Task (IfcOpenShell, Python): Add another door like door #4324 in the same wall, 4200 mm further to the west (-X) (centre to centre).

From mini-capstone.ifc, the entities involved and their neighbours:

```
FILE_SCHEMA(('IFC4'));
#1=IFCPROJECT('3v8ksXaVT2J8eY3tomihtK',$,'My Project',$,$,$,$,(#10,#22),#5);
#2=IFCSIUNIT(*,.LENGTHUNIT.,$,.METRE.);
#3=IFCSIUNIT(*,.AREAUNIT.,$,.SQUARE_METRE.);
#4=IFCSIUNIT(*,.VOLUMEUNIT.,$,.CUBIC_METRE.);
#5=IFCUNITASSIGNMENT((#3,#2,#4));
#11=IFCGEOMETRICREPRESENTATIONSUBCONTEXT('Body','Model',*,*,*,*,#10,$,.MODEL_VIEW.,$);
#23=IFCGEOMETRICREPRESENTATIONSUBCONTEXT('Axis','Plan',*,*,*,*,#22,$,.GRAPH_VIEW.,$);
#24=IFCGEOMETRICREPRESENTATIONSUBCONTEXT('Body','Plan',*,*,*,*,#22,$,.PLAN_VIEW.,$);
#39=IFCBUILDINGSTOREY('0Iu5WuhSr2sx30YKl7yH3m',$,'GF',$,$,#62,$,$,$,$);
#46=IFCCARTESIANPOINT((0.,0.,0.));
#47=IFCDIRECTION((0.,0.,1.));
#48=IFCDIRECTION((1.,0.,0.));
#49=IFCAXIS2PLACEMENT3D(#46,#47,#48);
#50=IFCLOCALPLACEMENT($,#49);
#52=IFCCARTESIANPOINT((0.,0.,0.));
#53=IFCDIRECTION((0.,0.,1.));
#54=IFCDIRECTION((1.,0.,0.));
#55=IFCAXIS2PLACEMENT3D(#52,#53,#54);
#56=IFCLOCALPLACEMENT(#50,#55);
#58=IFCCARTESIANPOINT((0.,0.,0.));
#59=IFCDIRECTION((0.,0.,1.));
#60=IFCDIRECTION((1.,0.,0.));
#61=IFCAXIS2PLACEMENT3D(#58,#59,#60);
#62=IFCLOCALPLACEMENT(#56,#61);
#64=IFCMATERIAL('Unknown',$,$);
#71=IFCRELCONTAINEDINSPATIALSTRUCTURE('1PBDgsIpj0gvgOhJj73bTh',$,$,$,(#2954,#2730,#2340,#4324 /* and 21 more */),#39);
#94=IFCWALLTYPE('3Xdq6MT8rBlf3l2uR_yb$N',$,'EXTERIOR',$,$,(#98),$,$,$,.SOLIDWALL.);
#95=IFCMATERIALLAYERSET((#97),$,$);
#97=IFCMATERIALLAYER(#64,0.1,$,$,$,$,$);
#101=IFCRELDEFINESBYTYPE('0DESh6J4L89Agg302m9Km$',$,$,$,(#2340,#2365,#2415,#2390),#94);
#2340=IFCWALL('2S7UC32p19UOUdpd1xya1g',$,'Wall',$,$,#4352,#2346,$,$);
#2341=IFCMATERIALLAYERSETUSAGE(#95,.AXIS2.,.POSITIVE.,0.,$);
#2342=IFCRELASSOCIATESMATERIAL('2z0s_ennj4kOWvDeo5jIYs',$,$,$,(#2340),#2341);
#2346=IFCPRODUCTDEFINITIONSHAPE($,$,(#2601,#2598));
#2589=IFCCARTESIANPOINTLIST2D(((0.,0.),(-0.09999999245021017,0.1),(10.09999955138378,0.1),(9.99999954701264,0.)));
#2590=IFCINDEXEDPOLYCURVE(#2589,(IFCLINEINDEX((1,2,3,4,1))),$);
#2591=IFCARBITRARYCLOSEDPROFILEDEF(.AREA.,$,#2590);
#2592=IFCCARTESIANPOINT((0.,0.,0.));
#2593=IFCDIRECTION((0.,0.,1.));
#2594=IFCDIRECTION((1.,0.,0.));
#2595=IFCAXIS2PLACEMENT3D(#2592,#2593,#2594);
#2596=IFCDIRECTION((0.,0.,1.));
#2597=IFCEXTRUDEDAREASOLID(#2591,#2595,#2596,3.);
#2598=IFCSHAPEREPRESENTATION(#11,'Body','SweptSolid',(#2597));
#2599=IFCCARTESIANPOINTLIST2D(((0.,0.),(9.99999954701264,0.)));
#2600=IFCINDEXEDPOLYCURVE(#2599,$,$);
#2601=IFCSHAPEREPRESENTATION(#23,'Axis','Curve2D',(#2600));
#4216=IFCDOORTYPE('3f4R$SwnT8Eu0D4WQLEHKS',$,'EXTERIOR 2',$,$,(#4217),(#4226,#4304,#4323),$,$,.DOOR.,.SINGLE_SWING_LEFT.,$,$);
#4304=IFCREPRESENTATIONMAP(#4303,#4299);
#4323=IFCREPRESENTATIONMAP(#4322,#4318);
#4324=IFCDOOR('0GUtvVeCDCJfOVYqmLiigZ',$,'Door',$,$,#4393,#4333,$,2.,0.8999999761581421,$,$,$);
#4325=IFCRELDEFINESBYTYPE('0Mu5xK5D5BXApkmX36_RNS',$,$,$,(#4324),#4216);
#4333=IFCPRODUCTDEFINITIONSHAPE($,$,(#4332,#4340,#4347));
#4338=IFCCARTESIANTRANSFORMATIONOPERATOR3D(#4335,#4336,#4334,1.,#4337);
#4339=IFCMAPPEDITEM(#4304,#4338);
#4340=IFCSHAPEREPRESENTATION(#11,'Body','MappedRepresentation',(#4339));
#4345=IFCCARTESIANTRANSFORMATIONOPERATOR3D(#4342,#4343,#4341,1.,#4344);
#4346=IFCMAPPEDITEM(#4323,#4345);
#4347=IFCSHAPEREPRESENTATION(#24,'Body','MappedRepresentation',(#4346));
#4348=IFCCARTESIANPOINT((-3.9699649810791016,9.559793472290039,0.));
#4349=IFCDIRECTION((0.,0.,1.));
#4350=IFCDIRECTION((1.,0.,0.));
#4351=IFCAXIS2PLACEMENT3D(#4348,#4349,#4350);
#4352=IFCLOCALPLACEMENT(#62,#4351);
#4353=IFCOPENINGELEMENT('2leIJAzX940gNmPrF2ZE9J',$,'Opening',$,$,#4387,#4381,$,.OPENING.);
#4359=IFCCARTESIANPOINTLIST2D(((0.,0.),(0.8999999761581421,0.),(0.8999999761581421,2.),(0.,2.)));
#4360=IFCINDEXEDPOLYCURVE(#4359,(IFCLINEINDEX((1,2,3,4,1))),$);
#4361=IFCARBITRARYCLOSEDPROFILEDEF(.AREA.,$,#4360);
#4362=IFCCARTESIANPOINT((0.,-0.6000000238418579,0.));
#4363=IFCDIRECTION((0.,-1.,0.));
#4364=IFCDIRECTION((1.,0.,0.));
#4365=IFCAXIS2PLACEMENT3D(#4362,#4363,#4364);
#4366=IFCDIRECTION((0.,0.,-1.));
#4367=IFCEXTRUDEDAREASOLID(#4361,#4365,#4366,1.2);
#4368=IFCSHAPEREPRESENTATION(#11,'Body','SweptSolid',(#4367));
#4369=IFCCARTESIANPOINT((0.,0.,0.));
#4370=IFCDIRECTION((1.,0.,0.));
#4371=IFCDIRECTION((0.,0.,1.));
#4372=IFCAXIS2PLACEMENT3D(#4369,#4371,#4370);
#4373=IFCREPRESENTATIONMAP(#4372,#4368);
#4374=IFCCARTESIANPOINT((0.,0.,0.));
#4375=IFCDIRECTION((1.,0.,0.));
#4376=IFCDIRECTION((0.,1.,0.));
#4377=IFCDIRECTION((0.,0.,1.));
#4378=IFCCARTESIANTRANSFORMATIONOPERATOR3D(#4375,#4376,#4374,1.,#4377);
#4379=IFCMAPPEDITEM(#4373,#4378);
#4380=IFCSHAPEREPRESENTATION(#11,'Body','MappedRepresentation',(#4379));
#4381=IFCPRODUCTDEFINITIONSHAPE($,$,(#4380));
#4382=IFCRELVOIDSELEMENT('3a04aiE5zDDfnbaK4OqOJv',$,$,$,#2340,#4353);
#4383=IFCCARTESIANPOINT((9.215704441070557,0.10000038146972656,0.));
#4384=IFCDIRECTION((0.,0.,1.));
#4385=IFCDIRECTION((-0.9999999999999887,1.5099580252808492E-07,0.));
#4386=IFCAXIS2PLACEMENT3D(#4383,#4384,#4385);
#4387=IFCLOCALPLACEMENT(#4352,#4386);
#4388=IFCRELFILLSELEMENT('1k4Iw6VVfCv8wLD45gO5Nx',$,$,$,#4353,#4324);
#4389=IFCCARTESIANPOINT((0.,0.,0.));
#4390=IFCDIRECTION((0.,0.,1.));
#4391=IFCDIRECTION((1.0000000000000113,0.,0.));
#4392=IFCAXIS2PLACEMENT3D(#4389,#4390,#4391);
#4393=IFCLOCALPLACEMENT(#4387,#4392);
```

```python
import ifcopenshell
import ifcopenshell.api.feature
import ifcopenshell.api.geometry
import ifcopenshell.api.root
import ifcopenshell.geom
import ifcopenshell.util.element
import ifcopenshell.util.placement
import ifcopenshell.util.shape

model = ifcopenshell.open("mini-capstone.ifc")
settings = ifcopenshell.geom.settings()


def volume(element):
    """Net volume in cubic metres, openings subtracted."""
    shape = ifcopenshell.geom.create_shape(settings, element)
    return ifcopenshell.util.shape.get_volume(shape.geometry)


door = model.by_id(4324)
opening = door.FillsVoids[0].RelatingOpeningElement
wall = opening.VoidsElements[0].RelatingBuildingElement
before = volume(wall)
shift = ifcopenshell.util.placement.get_local_placement(wall.ObjectPlacement)[:3, 0] * -4.2

# copy_class copies the void relationship, type, container and properties, but no geometry.
new_opening = ifcopenshell.api.root.copy_class(model, product=opening)
new_opening.Representation = ifcopenshell.util.element.copy_deep(
    model, opening.Representation, exclude=["IfcGeometricRepresentationContext", "IfcRepresentationMap"]
)
new_door = ifcopenshell.api.root.copy_class(model, product=door)
new_door.Representation = ifcopenshell.util.element.copy_deep(
    model, door.Representation, exclude=["IfcGeometricRepresentationContext", "IfcRepresentationMap"]
)
ifcopenshell.api.feature.add_filling(model, opening=new_opening, element=new_door)

for old, new in ((opening, new_opening), (door, new_door)):
    matrix = ifcopenshell.util.placement.get_local_placement(old.ObjectPlacement)
    matrix[:3, 3] += shift
    ifcopenshell.api.geometry.edit_object_placement(model, product=new, matrix=matrix, is_si=False)

after = volume(wall)

print(f"wall volume {before:.3f} -> {after:.3f} m3")

model.write("mini-capstone_v2.ifc")
```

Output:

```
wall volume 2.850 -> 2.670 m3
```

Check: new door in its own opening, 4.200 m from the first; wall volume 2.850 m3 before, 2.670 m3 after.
